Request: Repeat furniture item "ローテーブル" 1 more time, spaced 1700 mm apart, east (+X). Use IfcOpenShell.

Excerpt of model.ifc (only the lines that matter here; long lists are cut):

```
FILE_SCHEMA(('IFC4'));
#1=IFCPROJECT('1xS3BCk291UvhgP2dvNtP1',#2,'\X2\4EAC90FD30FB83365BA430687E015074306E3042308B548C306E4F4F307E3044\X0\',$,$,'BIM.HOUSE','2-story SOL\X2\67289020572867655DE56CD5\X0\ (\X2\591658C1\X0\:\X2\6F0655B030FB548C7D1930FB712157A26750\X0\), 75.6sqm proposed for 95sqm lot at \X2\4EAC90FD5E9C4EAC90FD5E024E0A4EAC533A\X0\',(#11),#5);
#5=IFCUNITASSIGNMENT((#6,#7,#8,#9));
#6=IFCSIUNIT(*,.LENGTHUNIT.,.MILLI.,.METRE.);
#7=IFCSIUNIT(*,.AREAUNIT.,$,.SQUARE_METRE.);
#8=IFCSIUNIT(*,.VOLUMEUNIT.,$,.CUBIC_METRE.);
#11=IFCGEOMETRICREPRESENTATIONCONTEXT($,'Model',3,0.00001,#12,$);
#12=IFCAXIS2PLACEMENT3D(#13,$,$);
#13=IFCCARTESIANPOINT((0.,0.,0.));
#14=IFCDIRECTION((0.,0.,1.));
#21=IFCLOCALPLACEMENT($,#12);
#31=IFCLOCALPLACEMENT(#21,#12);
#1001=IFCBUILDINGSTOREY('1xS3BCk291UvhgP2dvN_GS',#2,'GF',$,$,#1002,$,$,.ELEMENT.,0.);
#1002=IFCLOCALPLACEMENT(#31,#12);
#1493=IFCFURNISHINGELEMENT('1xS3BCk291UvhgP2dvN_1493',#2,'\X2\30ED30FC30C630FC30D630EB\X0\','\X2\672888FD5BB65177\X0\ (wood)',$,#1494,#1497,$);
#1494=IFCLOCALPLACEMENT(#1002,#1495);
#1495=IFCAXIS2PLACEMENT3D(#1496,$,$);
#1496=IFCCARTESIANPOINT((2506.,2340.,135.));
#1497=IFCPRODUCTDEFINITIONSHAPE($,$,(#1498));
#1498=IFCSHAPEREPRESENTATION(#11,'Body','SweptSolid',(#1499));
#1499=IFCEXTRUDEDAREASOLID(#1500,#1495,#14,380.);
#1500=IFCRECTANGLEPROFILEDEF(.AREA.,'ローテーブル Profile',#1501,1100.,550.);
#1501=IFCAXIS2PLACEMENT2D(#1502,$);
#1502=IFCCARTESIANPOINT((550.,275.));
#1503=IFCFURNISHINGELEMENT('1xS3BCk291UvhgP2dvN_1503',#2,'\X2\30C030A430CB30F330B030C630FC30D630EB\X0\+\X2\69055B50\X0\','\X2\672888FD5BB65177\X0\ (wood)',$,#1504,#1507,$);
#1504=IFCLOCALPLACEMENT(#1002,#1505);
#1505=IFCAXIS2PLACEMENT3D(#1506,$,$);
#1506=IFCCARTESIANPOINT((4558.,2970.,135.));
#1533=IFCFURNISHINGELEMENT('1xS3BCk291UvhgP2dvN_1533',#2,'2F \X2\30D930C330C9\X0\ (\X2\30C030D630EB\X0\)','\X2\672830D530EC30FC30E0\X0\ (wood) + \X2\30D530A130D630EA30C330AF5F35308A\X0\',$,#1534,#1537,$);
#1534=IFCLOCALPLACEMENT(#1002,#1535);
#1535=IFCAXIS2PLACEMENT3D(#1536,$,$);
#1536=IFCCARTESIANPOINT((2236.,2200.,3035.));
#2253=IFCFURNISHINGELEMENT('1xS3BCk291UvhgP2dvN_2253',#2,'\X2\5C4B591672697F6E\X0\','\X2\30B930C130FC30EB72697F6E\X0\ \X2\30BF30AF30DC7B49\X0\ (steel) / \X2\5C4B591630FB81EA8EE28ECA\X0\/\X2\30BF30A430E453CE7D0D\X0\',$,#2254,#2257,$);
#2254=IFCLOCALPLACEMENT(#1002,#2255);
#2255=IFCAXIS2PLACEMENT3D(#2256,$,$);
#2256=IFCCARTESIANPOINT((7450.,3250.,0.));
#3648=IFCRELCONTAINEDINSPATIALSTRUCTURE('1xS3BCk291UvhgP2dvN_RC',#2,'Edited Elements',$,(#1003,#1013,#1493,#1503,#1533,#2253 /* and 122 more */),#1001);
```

```python
import numpy as np
import ifcopenshell
import ifcopenshell.api.geometry
import ifcopenshell.api.root
import ifcopenshell.util.element
import ifcopenshell.util.placement
import ifcopenshell.util.unit

model = ifcopenshell.open("model.ifc")
unit_scale = ifcopenshell.util.unit.calculate_unit_scale(model)


def reuse_history(source, copy):
    """copy_class also copies each property set's owner history, people and application; keep the originals."""
    for rel in copy.IsDefinedBy:
        if rel.is_a("IfcRelDefinesByProperties") and (history := rel.RelatingPropertyDefinition.OwnerHistory):
            rel.RelatingPropertyDefinition.OwnerHistory = source.OwnerHistory
            ifcopenshell.util.element.remove_deep2(model, history)


source = model.by_id(1493)
base = ifcopenshell.util.placement.get_local_placement(source.ObjectPlacement)
step = np.array([1.0, 0.0, 0.0]) * 1.7 / unit_scale

for i in range(1, 2):
    copy = ifcopenshell.api.root.copy_class(model, product=source)
    copy.Representation = ifcopenshell.util.element.copy_deep(
        model, source.Representation, exclude=["IfcGeometricRepresentationContext", "IfcRepresentationMap"]
    )
    reuse_history(source, copy)
    matrix = base.copy()
    matrix[:3, 3] += i * step
    print("added at", matrix[:3, 3].round(3) + 0.0)
    ifcopenshell.api.geometry.edit_object_placement(model, product=copy, matrix=matrix, is_si=False)

model.write("model_v2.ifc")
```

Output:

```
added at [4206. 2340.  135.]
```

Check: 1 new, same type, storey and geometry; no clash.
